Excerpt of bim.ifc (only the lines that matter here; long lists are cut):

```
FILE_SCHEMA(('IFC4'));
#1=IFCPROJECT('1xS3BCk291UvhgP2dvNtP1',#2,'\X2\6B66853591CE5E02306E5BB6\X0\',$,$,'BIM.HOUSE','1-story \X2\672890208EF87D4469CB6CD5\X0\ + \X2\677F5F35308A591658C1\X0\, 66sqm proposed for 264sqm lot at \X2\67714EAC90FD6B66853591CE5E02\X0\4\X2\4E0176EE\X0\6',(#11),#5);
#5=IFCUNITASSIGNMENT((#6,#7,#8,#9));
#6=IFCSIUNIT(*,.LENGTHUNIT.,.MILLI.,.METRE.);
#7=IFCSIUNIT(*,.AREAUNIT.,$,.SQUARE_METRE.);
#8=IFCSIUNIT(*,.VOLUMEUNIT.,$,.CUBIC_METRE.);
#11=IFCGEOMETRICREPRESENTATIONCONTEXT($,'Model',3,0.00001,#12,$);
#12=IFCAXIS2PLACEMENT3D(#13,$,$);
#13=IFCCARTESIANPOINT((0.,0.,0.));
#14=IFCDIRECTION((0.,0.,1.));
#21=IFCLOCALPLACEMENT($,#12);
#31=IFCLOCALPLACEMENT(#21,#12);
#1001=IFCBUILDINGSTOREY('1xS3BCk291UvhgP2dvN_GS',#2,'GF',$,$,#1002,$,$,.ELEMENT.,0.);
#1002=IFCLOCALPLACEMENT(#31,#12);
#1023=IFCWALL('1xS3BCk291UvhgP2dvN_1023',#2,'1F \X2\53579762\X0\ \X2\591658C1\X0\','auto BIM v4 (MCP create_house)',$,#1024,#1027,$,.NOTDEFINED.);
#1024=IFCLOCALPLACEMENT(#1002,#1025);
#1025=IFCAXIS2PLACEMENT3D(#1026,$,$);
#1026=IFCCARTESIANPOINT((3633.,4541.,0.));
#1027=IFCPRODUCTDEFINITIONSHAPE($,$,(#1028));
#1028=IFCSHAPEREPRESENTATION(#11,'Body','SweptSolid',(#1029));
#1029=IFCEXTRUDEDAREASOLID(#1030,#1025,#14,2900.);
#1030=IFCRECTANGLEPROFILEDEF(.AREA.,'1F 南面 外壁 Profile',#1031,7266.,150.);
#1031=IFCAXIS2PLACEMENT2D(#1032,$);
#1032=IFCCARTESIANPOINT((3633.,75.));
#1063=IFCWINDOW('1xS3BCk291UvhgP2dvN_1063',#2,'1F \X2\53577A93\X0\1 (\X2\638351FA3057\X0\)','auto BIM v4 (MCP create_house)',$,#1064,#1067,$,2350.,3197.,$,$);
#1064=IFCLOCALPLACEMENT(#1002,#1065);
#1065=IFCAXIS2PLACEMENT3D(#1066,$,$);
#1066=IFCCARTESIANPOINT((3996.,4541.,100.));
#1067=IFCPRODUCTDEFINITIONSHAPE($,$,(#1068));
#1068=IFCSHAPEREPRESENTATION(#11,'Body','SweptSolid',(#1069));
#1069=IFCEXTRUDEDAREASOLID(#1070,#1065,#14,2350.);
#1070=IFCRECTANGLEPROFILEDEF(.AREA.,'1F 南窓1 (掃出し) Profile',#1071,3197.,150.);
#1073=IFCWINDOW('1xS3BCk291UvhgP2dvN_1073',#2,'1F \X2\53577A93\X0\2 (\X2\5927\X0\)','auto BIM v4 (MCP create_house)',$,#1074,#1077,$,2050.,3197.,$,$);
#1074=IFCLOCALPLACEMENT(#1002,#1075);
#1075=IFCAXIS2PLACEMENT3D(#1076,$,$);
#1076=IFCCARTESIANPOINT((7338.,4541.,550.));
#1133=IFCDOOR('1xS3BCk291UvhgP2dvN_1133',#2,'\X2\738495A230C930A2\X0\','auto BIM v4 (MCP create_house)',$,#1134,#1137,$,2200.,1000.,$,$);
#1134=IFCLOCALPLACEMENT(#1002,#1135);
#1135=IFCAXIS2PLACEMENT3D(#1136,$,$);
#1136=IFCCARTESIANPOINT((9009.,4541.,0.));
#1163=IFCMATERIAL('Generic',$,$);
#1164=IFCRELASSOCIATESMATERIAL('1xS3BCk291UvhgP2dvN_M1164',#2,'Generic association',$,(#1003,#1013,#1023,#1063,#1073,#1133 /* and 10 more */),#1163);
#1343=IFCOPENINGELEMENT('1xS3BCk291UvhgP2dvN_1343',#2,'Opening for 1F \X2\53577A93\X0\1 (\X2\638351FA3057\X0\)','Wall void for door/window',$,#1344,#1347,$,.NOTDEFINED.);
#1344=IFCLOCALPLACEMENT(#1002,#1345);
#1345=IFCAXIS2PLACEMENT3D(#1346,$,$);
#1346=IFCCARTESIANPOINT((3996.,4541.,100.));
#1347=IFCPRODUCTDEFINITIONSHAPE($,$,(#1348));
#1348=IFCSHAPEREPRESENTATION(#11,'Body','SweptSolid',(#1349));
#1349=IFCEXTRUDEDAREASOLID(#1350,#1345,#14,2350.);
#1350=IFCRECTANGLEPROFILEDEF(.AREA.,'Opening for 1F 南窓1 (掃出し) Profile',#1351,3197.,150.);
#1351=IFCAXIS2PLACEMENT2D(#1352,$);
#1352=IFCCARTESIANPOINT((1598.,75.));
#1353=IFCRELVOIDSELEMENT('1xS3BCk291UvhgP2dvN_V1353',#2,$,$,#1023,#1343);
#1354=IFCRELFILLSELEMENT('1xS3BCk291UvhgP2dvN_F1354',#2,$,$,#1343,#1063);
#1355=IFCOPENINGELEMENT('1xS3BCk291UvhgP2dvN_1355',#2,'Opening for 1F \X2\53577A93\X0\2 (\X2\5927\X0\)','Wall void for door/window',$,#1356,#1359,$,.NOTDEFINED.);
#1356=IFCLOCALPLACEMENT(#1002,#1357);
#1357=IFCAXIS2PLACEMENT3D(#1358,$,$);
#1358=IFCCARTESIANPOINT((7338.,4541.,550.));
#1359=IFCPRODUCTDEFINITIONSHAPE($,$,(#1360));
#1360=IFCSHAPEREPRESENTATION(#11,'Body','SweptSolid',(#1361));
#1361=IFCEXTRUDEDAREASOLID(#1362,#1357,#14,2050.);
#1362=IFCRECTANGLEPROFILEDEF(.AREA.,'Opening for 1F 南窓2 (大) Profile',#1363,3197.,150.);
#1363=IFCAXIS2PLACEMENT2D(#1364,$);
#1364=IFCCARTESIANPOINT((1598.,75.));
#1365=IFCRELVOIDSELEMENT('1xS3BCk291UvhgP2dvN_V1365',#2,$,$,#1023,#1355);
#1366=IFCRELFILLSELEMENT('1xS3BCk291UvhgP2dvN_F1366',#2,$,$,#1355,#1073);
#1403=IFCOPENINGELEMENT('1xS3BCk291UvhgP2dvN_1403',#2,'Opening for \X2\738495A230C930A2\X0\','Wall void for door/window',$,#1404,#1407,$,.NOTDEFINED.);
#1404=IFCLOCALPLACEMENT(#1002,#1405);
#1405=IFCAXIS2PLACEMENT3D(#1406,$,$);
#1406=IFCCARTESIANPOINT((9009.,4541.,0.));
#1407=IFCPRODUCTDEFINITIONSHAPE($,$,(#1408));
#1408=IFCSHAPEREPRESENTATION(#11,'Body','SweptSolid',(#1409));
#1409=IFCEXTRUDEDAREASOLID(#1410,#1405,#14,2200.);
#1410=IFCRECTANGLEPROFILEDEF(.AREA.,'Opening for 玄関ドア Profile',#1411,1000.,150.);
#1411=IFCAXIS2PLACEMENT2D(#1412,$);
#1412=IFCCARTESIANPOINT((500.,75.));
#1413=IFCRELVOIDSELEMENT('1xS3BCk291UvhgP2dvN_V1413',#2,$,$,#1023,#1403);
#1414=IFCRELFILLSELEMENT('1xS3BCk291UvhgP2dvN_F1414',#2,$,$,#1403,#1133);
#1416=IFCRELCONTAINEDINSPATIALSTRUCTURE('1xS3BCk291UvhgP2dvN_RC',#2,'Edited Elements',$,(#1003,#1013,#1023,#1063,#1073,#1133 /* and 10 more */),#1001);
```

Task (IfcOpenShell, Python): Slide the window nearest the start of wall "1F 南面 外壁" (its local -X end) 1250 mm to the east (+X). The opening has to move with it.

```python
import ifcopenshell
import ifcopenshell.api.geometry
import ifcopenshell.util.placement
import ifcopenshell.util.unit

model = ifcopenshell.open("bim.ifc")
unit_scale = ifcopenshell.util.unit.calculate_unit_scale(model)

window = model.by_id(1063)
opening = window.FillsVoids[0].RelatingOpeningElement
wall = opening.VoidsElements[0].RelatingBuildingElement

wall_matrix = ifcopenshell.util.placement.get_local_placement(wall.ObjectPlacement)
shift = wall_matrix[:3, 0] * 1.25 / unit_scale
before = ifcopenshell.util.placement.get_local_placement(window.ObjectPlacement)[:3, 3].copy()

# The window is not placed relative to its opening, so move both.
for product in (opening, window):
    matrix = ifcopenshell.util.placement.get_local_placement(product.ObjectPlacement)
    matrix[:3, 3] += shift
    ifcopenshell.api.geometry.edit_object_placement(model, product=product, matrix=matrix, is_si=False)

after = ifcopenshell.util.placement.get_local_placement(window.ObjectPlacement)[:3, 3]
print("window moved by", (after - before).round(3) + 0.0)

model.write("bim_updated.ifc")
```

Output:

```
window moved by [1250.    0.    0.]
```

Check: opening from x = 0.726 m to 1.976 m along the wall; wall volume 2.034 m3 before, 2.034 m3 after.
